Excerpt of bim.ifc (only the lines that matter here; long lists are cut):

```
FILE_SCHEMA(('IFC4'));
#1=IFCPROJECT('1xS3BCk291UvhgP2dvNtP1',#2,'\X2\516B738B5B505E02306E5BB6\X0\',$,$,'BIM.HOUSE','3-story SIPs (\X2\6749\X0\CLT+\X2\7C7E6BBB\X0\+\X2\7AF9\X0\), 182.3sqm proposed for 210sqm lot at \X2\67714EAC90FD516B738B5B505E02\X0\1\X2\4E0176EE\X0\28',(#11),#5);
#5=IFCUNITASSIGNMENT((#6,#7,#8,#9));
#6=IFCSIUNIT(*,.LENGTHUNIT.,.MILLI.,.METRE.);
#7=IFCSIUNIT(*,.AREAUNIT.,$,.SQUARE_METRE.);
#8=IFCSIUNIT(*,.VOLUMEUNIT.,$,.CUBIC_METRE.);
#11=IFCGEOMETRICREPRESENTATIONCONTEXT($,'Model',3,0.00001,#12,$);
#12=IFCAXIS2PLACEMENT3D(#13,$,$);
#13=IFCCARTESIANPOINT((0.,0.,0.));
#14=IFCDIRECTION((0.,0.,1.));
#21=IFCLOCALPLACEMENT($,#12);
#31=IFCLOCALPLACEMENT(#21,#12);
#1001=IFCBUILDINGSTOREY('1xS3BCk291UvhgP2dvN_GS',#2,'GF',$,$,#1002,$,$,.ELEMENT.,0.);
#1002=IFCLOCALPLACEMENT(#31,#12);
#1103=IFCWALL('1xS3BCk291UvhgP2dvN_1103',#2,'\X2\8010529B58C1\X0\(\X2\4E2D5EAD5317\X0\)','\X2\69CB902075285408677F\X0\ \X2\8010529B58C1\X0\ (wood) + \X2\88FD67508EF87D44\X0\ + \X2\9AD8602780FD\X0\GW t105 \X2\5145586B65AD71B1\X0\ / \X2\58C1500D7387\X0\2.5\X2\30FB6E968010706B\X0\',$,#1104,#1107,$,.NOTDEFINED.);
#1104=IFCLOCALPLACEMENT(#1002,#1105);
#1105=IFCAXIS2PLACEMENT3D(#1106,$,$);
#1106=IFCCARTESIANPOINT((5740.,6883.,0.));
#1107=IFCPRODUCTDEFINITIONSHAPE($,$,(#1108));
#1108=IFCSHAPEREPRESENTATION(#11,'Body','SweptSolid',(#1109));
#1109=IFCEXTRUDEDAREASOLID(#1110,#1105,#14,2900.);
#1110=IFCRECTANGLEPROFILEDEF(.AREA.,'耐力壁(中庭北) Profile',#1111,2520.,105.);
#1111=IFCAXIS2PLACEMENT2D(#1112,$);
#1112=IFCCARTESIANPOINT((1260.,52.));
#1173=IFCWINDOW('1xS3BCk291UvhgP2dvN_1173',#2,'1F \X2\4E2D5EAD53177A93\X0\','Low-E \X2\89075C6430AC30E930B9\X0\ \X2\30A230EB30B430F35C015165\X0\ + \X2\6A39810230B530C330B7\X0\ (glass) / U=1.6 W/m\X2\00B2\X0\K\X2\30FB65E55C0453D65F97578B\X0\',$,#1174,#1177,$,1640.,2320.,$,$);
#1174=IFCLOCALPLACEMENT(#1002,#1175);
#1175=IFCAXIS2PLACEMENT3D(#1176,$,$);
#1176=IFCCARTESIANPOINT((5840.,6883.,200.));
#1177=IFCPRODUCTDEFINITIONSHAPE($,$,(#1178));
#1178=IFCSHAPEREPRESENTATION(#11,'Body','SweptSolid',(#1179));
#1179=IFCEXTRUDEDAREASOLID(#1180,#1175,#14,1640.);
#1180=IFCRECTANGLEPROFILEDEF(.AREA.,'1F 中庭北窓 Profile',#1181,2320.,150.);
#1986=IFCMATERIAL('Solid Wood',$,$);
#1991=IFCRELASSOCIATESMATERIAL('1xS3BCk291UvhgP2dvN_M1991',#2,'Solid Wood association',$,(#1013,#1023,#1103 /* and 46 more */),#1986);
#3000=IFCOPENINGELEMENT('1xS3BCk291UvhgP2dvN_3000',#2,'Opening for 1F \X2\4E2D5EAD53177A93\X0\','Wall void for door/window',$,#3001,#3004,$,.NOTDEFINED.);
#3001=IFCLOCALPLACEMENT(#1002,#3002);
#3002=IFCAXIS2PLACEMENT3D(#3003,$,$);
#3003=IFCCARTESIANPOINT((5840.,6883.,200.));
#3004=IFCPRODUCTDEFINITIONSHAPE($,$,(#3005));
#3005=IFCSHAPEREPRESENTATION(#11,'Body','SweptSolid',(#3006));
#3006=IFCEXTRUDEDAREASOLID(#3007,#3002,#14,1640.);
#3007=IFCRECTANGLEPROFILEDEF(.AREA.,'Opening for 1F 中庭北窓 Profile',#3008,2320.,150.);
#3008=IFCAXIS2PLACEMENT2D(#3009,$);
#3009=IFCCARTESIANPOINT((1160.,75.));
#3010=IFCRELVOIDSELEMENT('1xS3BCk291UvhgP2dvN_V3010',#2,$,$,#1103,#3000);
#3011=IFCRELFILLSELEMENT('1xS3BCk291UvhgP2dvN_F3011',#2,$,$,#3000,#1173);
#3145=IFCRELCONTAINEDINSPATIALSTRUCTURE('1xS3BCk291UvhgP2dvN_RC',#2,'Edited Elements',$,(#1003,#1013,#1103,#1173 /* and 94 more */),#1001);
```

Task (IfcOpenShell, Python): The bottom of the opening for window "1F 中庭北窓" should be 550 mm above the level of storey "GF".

```python
import numpy as np
import ifcopenshell
import ifcopenshell.api.geometry
import ifcopenshell.geom
import ifcopenshell.util.element
import ifcopenshell.util.placement
import ifcopenshell.util.shape
import ifcopenshell.util.unit

model = ifcopenshell.open("bim.ifc")
unit_scale = ifcopenshell.util.unit.calculate_unit_scale(model)

window = model.by_guid("1xS3BCk291UvhgP2dvN_1173")
opening = window.FillsVoids[0].RelatingOpeningElement
storey = ifcopenshell.util.element.get_container(window, ifc_class="IfcBuildingStorey")
level = ifcopenshell.util.placement.get_local_placement(storey.ObjectPlacement)[2, 3]

# The opening's origin need not be at the sill, so measure its lowest point.
shape = ifcopenshell.geom.create_shape(ifcopenshell.geom.settings(), opening)
bottom = ifcopenshell.util.shape.get_shape_bottom_elevation(shape, shape.geometry) / unit_scale
dz = level + 0.55 / unit_scale - bottom

shift = np.array([0.0, 0.0, dz])
# The window is not placed relative to its opening, so move both.
for product in (opening, window):
    matrix = ifcopenshell.util.placement.get_local_placement(product.ObjectPlacement)
    matrix[:3, 3] += shift
    ifcopenshell.api.geometry.edit_object_placement(model, product=product, matrix=matrix, is_si=False)

print(f"moved by {dz * unit_scale:+.3f} m")

model.write("bim_updated.ifc")
```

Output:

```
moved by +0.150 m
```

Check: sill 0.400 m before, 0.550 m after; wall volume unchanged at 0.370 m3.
